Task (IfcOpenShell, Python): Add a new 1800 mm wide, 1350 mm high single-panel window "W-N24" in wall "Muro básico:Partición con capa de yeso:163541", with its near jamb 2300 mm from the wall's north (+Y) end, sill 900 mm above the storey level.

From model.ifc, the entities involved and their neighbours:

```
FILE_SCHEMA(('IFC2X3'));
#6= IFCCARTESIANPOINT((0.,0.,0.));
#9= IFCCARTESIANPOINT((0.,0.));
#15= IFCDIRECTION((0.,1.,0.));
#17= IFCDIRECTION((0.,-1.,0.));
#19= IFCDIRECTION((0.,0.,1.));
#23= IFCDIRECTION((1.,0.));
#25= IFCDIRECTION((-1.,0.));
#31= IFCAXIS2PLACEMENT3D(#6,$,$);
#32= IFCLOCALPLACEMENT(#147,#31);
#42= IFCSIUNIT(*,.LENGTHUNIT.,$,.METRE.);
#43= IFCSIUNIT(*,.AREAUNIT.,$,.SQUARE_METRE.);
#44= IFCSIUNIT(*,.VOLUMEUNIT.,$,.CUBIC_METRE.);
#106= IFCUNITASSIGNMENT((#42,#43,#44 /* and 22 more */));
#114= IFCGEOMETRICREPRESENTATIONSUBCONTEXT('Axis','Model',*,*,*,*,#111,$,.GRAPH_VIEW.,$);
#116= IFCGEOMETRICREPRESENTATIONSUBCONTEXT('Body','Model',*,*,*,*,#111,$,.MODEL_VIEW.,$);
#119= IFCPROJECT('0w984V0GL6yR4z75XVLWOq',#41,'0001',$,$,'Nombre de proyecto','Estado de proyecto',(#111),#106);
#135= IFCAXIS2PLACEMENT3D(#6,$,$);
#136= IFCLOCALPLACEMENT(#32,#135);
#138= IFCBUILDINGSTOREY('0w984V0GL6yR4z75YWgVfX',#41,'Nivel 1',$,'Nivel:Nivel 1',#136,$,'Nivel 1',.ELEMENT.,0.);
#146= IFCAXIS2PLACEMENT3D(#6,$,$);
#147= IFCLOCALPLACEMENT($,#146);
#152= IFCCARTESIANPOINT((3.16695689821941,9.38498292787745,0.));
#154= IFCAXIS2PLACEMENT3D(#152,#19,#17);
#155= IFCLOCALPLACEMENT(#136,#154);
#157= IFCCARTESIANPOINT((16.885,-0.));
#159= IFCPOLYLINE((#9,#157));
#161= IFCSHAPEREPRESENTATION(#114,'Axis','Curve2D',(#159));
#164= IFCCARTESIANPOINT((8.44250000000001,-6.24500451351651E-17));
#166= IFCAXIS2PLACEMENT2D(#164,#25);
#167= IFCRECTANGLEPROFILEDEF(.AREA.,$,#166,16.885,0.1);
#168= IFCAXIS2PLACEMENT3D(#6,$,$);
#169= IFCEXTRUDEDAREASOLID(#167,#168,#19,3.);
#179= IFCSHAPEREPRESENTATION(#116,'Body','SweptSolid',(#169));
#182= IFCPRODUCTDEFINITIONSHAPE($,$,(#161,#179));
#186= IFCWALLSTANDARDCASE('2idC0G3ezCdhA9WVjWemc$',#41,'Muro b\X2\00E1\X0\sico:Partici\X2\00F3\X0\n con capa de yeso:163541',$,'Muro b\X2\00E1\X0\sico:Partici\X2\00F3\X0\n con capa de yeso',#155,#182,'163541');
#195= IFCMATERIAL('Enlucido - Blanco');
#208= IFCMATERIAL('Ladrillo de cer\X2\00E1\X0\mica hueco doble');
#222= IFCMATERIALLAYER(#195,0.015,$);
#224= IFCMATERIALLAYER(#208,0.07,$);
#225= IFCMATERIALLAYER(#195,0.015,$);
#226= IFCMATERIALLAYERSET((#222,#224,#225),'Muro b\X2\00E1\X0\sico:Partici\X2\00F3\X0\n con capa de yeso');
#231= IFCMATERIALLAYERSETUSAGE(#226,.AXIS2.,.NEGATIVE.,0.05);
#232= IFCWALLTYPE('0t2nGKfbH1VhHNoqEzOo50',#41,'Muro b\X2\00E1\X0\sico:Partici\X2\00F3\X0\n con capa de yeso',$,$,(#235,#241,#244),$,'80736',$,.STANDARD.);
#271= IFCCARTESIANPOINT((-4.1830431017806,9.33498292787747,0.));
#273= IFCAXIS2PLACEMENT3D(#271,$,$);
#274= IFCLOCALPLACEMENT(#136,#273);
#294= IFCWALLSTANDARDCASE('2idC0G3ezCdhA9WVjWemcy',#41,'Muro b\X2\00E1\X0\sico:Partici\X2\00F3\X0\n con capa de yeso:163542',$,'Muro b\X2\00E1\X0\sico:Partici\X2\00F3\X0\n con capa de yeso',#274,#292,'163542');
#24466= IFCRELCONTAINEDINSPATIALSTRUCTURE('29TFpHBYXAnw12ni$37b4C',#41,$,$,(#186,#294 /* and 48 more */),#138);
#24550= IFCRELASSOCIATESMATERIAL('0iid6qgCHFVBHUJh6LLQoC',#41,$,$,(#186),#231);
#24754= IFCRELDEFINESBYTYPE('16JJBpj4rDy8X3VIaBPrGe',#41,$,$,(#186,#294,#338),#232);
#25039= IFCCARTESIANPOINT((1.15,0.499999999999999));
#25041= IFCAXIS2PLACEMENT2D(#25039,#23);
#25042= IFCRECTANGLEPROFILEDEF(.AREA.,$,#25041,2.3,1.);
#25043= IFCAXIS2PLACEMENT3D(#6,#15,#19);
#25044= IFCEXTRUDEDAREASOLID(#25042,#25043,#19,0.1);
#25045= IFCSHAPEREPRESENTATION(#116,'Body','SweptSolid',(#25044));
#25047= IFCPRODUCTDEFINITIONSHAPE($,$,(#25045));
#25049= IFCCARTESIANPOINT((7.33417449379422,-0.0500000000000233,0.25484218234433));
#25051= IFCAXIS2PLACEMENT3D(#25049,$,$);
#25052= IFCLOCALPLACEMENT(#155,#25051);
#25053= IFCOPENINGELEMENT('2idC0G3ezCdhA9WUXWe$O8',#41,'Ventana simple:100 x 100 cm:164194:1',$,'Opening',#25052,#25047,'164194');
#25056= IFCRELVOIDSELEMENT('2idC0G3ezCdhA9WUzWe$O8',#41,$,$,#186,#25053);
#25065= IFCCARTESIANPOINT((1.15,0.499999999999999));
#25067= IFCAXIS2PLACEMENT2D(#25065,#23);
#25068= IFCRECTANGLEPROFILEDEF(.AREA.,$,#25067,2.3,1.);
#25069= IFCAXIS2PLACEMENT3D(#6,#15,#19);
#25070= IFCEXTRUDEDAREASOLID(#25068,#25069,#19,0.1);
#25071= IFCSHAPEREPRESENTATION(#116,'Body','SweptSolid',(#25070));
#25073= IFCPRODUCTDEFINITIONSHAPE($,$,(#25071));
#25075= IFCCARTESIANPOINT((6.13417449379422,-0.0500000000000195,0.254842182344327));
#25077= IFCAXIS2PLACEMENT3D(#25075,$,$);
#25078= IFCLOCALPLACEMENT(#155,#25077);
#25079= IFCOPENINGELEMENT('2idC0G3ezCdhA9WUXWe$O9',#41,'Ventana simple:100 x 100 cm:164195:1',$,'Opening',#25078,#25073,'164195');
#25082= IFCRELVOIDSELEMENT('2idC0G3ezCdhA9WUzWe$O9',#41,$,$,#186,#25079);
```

```python
import numpy as np
import ifcopenshell
import ifcopenshell.api.feature
import ifcopenshell.api.geometry
import ifcopenshell.api.root
import ifcopenshell.api.spatial
import ifcopenshell.api.type
import ifcopenshell.geom
import ifcopenshell.util.element
import ifcopenshell.util.placement
import ifcopenshell.util.representation
import ifcopenshell.util.shape
import ifcopenshell.util.unit

model = ifcopenshell.open("model.ifc")
unit_scale = ifcopenshell.util.unit.calculate_unit_scale(model)
settings = ifcopenshell.geom.settings()


def volume(element):
    """Net volume in cubic metres, openings subtracted."""
    shape = ifcopenshell.geom.create_shape(settings, element)
    return ifcopenshell.util.shape.get_volume(shape.geometry)


wall = model.by_guid("2idC0G3ezCdhA9WVjWemc$")
storey = ifcopenshell.util.element.get_container(wall, ifc_class="IfcBuildingStorey")
context = ifcopenshell.util.representation.get_context(model, "Model", "Body", "MODEL_VIEW")
before = volume(wall)

width, height, from_end, sill = 1.8, 1.35, 2.3, 0.9  # metres

# The wall runs along its own X axis, and the end named is its -X end.
wall_shape = ifcopenshell.geom.create_shape(settings, wall)
x, y, z = ifcopenshell.util.shape.get_vertices(wall_shape.geometry).T
start = x.min() + from_end
face, thickness = float(y.min()), float(y.max() - y.min())
wall_matrix = ifcopenshell.util.placement.get_local_placement(wall.ObjectPlacement)
level = ifcopenshell.util.placement.get_local_placement(storey.ObjectPlacement)[2, 3]


def in_wall(x, y):
    """Placement at x, y metres in the wall's axes, at sill height."""
    matrix = wall_matrix.copy()
    matrix[:, 3] = wall_matrix @ np.array([x / unit_scale, y / unit_scale, 0.0, 1.0])
    matrix[2, 3] = level + sill / unit_scale
    return matrix


# Opening: a box that overshoots both wall faces by 50 mm.
opening = ifcopenshell.api.root.create_entity(model, ifc_class="IfcOpeningElement")
box = ifcopenshell.api.geometry.add_wall_representation(
    model, context=context, length=width, height=height, thickness=thickness + 0.1
)
ifcopenshell.api.geometry.assign_representation(model, product=opening, representation=box)
ifcopenshell.api.geometry.edit_object_placement(model, product=opening, matrix=in_wall(start, face - 0.05), is_si=False)
ifcopenshell.api.feature.add_feature(model, feature=opening, element=wall)

window = ifcopenshell.api.root.create_entity(model, ifc_class="IfcWindow", name="W-N24")
window.OverallWidth, window.OverallHeight = width / unit_scale, height / unit_scale
body = ifcopenshell.api.geometry.add_window_representation(
    model,
    context=context,
    overall_width=window.OverallWidth,
    overall_height=window.OverallHeight,
    partition_type="SINGLE_PANEL",
)
ifcopenshell.api.geometry.assign_representation(model, product=window, representation=body)
ifcopenshell.api.spatial.assign_container(model, products=[window], relating_structure=storey)
fills = ifcopenshell.api.feature.add_filling(model, opening=opening, element=window)
fills.OwnerHistory = window.OwnerHistory  # required in IFC2X3

# IFC2X3 keeps the operation on the window style.
style = ifcopenshell.api.root.create_entity(model, ifc_class="IfcWindowStyle", name="W-N24")
style.OperationType, style.ConstructionType = "SINGLE_PANEL", "NOTDEFINED"
style.ParameterTakesPrecedence = style.Sizeable = False
ifcopenshell.api.type.assign_type(model, related_objects=[window], relating_type=style)

# Centre the window in the wall's thickness.
ifcopenshell.api.geometry.edit_object_placement(model, product=window, matrix=in_wall(start, face), is_si=False)
window_shape = ifcopenshell.geom.create_shape(settings, window)
depth = ifcopenshell.util.shape.get_vertices(window_shape.geometry)[:, 1]
offset = face + thickness / 2 - (depth.min() + depth.max()) / 2
ifcopenshell.api.geometry.edit_object_placement(model, product=window, matrix=in_wall(start, offset), is_si=False)

after = volume(wall)

print(f"wall volume {before:.3f} -> {after:.3f} m3")

model.write("model_v2.ifc")
```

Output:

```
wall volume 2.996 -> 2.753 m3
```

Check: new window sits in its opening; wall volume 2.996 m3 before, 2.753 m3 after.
